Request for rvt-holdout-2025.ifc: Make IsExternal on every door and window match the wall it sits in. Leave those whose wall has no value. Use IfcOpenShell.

First a look at what the model holds.

```python
import ifcopenshell
import ifcopenshell.util.element

model = ifcopenshell.open("rvt-holdout-2025.ifc")
print(model.schema)
seen = {}
for e in model.by_type("IfcDoor") + model.by_type("IfcWindow"):
    if not e.FillsVoids:
        continue
    host = e.FillsVoids[0].RelatingOpeningElement.VoidsElements[0].RelatingBuildingElement
    own = ifcopenshell.util.element.get_pset(e, f"Pset_{e.is_a()[3:].removesuffix('StandardCase')}Common", "IsExternal")
    wall = ifcopenshell.util.element.get_pset(host, "Pset_WallCommon", "IsExternal")
    seen[e.is_a(), own, wall] = seen.get((e.is_a(), own, wall), 0) + 1
for (cls, own, wall), count in sorted(seen.items(), key=str):
    print(count, cls, "IsExternal:", own, "| host wall:", wall)
```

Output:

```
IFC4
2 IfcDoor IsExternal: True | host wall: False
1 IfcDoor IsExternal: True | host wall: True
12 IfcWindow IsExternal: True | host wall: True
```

```python
import ifcopenshell
import ifcopenshell.api.pset
import ifcopenshell.util.element

model = ifcopenshell.open("rvt-holdout-2025.ifc")

count = 0
for ifc_class, pset_name in (("IfcDoor", "Pset_DoorCommon"), ("IfcWindow", "Pset_WindowCommon")):
    for e in model.by_type(ifc_class):
        if not e.FillsVoids:
            continue
        host = e.FillsVoids[0].RelatingOpeningElement.VoidsElements[0].RelatingBuildingElement
        external = ifcopenshell.util.element.get_pset(host, "Pset_WallCommon", "IsExternal")
        if external is None or ifcopenshell.util.element.get_pset(e, pset_name, "IsExternal") == external:
            continue
        pset = ifcopenshell.api.pset.add_pset(model, product=e, name=pset_name)
        ifcopenshell.api.pset.edit_pset(model, pset=pset, properties={"IsExternal": external})
        count += 1

print(count, "updated")

model.write("rvt-holdout-2025_v2.ifc")
```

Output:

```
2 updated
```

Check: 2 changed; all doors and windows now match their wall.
